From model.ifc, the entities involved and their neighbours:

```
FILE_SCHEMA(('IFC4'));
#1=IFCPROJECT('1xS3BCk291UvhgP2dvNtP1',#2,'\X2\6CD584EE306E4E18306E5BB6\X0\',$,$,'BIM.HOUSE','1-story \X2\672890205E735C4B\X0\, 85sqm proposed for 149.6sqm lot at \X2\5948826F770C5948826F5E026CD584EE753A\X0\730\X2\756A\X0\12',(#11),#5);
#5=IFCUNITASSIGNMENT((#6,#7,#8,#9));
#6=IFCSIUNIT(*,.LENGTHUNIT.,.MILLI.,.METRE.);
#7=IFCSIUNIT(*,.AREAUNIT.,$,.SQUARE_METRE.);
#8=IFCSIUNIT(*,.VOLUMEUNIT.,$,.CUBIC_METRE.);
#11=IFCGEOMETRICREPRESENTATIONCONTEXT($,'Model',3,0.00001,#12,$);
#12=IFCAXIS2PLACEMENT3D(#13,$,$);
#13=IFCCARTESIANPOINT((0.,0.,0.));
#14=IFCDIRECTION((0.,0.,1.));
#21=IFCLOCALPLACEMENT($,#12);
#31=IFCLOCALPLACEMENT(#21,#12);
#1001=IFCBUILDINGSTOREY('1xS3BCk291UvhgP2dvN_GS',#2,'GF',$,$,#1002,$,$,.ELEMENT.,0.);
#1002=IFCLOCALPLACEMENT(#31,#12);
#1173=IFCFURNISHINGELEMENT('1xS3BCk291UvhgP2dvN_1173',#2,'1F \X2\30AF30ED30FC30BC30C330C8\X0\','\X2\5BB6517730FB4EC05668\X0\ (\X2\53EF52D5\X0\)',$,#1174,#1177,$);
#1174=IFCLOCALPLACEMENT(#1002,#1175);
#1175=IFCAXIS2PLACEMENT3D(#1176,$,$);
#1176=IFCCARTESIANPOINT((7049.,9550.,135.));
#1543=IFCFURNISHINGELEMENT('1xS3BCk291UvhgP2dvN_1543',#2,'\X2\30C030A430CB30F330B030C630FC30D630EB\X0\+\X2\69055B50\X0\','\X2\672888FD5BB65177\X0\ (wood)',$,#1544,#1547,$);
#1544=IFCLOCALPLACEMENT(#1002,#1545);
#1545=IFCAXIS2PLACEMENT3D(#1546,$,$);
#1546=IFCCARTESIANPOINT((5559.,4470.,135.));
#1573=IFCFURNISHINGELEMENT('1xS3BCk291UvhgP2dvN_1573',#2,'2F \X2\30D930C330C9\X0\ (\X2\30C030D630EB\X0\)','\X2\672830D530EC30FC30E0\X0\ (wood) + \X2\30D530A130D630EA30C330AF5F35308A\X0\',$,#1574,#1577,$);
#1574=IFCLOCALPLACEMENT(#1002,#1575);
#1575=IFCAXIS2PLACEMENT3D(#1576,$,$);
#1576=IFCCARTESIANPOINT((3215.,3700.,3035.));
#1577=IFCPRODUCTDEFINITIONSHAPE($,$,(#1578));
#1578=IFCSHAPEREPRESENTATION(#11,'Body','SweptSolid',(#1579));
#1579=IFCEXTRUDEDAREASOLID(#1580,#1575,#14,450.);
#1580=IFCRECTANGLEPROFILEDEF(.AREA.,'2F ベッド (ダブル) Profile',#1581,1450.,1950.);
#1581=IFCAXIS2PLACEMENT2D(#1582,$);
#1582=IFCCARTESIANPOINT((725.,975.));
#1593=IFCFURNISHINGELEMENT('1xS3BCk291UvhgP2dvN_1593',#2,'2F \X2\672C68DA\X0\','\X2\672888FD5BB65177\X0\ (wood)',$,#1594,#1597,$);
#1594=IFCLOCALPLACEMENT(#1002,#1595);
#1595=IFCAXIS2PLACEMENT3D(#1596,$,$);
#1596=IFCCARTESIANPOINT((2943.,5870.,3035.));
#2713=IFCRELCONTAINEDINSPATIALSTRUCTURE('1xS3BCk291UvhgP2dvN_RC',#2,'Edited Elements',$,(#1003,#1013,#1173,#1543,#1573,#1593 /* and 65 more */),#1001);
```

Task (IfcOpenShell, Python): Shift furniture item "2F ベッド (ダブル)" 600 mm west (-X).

```python
import ifcopenshell
import ifcopenshell.api.geometry
import ifcopenshell.util.placement
import ifcopenshell.util.unit

model = ifcopenshell.open("model.ifc")
unit_scale = ifcopenshell.util.unit.calculate_unit_scale(model)

item = model.by_guid("1xS3BCk291UvhgP2dvN_1573")
matrix = ifcopenshell.util.placement.get_local_placement(item.ObjectPlacement)
matrix[0, 3] -= 0.6 / unit_scale
ifcopenshell.api.geometry.edit_object_placement(model, product=item, matrix=matrix, is_si=False)

print(ifcopenshell.util.placement.get_local_placement(item.ObjectPlacement).round(3) + 0.0)

model.write("model_updated.ifc")
```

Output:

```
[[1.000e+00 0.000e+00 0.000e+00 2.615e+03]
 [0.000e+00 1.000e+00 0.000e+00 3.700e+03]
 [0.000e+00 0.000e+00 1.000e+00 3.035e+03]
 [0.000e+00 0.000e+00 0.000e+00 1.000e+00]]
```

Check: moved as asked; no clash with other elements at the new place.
